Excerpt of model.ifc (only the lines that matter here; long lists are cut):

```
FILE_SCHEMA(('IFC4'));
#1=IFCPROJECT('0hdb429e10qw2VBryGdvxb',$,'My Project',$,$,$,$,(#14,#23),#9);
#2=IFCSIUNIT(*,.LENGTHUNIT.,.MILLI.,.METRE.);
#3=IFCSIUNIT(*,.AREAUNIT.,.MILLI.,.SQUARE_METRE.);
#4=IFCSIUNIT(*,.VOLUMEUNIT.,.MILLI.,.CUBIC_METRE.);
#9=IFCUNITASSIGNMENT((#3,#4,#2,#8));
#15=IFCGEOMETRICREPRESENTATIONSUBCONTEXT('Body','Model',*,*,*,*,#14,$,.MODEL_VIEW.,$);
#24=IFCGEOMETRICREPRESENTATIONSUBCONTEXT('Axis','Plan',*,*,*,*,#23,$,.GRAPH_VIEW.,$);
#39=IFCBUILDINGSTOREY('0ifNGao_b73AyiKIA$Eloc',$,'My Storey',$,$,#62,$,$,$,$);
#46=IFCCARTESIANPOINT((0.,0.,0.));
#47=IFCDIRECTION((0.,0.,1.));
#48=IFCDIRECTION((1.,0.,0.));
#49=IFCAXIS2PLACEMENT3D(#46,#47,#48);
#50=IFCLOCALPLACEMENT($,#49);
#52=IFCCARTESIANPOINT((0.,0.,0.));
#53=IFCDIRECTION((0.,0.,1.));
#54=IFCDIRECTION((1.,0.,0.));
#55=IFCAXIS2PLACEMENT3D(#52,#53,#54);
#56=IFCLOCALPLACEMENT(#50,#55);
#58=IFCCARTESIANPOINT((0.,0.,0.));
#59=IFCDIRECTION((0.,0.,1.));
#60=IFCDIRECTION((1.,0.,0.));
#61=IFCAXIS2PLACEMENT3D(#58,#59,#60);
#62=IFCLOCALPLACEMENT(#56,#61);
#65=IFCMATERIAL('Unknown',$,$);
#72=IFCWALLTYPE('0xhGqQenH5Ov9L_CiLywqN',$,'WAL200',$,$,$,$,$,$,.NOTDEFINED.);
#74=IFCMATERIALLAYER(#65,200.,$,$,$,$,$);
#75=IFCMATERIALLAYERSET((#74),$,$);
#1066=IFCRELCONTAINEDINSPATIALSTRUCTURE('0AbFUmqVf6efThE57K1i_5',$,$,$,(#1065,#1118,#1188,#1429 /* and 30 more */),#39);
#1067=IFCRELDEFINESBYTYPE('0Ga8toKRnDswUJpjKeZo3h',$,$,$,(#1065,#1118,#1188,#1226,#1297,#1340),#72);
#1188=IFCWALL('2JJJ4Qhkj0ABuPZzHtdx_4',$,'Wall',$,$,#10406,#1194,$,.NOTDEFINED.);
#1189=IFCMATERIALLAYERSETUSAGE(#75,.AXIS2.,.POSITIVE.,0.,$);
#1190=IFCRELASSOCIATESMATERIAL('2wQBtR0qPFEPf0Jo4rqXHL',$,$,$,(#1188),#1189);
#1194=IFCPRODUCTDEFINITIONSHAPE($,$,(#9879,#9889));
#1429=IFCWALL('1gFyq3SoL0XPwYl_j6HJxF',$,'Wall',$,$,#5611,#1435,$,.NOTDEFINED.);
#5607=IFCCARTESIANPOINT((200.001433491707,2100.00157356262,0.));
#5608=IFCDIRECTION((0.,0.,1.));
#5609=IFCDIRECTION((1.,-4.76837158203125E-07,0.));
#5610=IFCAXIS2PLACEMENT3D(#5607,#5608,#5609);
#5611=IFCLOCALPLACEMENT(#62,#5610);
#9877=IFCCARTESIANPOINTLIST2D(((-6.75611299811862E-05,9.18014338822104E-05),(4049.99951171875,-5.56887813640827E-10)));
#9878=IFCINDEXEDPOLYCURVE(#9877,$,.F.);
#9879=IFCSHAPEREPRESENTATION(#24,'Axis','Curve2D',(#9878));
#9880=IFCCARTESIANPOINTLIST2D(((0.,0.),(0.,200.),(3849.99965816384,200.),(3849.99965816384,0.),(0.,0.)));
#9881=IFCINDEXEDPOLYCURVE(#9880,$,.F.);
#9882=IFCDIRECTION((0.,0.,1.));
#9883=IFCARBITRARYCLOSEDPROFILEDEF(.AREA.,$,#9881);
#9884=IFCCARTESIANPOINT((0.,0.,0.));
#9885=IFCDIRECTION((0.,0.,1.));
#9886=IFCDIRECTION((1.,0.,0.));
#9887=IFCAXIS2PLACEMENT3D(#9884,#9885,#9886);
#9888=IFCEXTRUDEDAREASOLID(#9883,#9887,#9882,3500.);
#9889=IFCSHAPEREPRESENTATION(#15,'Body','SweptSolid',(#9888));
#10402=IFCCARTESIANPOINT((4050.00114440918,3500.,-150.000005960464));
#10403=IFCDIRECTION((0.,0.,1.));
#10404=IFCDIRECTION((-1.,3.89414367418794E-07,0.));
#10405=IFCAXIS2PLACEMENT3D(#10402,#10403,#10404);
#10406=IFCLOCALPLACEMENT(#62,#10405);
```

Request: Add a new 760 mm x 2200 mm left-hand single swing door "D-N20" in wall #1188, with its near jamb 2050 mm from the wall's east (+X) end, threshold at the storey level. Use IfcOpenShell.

```python
import numpy as np
import ifcopenshell
import ifcopenshell.api.feature
import ifcopenshell.api.geometry
import ifcopenshell.api.root
import ifcopenshell.api.spatial
import ifcopenshell.geom
import ifcopenshell.util.element
import ifcopenshell.util.placement
import ifcopenshell.util.representation
import ifcopenshell.util.shape
import ifcopenshell.util.unit

model = ifcopenshell.open("model.ifc")
unit_scale = ifcopenshell.util.unit.calculate_unit_scale(model)
settings = ifcopenshell.geom.settings()


def volume(element):
    """Net volume in cubic metres, openings subtracted."""
    shape = ifcopenshell.geom.create_shape(settings, element)
    return ifcopenshell.util.shape.get_volume(shape.geometry)


wall = model.by_id(1188)
storey = ifcopenshell.util.element.get_container(wall, ifc_class="IfcBuildingStorey")
context = ifcopenshell.util.representation.get_context(model, "Model", "Body", "MODEL_VIEW")
before = volume(wall)

width, height, from_end, sill = 0.76, 2.2, 2.05, 0.0  # metres

# The wall runs along its own X axis, and the end named is its -X end.
wall_shape = ifcopenshell.geom.create_shape(settings, wall)
x, y, z = ifcopenshell.util.shape.get_vertices(wall_shape.geometry).T
start = x.min() + from_end
face, thickness = float(y.min()), float(y.max() - y.min())
wall_matrix = ifcopenshell.util.placement.get_local_placement(wall.ObjectPlacement)
level = ifcopenshell.util.placement.get_local_placement(storey.ObjectPlacement)[2, 3]


def in_wall(x, y):
    """Placement at x, y metres in the wall's axes, at sill height."""
    matrix = wall_matrix.copy()
    matrix[:, 3] = wall_matrix @ np.array([x / unit_scale, y / unit_scale, 0.0, 1.0])
    matrix[2, 3] = level + sill / unit_scale
    return matrix


# Opening: a box that overshoots both wall faces by 50 mm.
opening = ifcopenshell.api.root.create_entity(model, ifc_class="IfcOpeningElement", predefined_type="OPENING")
box = ifcopenshell.api.geometry.add_wall_representation(
    model, context=context, length=width, height=height, thickness=thickness + 0.1
)
ifcopenshell.api.geometry.assign_representation(model, product=opening, representation=box)
ifcopenshell.api.geometry.edit_object_placement(model, product=opening, matrix=in_wall(start, face - 0.05), is_si=False)
ifcopenshell.api.feature.add_feature(model, feature=opening, element=wall)

door = ifcopenshell.api.root.create_entity(model, ifc_class="IfcDoor", name="D-N20", predefined_type="DOOR")
door.OverallWidth, door.OverallHeight = width / unit_scale, height / unit_scale
door.OperationType = "SINGLE_SWING_LEFT"
body = ifcopenshell.api.geometry.add_door_representation(
    model,
    context=context,
    overall_width=door.OverallWidth,
    overall_height=door.OverallHeight,
    operation_type="SINGLE_SWING_LEFT",
    lining_properties={"LiningDepth": thickness / unit_scale, "ThresholdDepth": thickness / unit_scale},
)
ifcopenshell.api.geometry.assign_representation(model, product=door, representation=body)
ifcopenshell.api.spatial.assign_container(model, products=[door], relating_structure=storey)
ifcopenshell.api.feature.add_filling(model, opening=opening, element=door)

# The lining spans the wall, so the door starts at the wall face.
ifcopenshell.api.geometry.edit_object_placement(model, product=door, matrix=in_wall(start, face), is_si=False)

after = volume(wall)

print(f"wall volume {before:.3f} -> {after:.3f} m3")

model.write("model_edited.ifc")
```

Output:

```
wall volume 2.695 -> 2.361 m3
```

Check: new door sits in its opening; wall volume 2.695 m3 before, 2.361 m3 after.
